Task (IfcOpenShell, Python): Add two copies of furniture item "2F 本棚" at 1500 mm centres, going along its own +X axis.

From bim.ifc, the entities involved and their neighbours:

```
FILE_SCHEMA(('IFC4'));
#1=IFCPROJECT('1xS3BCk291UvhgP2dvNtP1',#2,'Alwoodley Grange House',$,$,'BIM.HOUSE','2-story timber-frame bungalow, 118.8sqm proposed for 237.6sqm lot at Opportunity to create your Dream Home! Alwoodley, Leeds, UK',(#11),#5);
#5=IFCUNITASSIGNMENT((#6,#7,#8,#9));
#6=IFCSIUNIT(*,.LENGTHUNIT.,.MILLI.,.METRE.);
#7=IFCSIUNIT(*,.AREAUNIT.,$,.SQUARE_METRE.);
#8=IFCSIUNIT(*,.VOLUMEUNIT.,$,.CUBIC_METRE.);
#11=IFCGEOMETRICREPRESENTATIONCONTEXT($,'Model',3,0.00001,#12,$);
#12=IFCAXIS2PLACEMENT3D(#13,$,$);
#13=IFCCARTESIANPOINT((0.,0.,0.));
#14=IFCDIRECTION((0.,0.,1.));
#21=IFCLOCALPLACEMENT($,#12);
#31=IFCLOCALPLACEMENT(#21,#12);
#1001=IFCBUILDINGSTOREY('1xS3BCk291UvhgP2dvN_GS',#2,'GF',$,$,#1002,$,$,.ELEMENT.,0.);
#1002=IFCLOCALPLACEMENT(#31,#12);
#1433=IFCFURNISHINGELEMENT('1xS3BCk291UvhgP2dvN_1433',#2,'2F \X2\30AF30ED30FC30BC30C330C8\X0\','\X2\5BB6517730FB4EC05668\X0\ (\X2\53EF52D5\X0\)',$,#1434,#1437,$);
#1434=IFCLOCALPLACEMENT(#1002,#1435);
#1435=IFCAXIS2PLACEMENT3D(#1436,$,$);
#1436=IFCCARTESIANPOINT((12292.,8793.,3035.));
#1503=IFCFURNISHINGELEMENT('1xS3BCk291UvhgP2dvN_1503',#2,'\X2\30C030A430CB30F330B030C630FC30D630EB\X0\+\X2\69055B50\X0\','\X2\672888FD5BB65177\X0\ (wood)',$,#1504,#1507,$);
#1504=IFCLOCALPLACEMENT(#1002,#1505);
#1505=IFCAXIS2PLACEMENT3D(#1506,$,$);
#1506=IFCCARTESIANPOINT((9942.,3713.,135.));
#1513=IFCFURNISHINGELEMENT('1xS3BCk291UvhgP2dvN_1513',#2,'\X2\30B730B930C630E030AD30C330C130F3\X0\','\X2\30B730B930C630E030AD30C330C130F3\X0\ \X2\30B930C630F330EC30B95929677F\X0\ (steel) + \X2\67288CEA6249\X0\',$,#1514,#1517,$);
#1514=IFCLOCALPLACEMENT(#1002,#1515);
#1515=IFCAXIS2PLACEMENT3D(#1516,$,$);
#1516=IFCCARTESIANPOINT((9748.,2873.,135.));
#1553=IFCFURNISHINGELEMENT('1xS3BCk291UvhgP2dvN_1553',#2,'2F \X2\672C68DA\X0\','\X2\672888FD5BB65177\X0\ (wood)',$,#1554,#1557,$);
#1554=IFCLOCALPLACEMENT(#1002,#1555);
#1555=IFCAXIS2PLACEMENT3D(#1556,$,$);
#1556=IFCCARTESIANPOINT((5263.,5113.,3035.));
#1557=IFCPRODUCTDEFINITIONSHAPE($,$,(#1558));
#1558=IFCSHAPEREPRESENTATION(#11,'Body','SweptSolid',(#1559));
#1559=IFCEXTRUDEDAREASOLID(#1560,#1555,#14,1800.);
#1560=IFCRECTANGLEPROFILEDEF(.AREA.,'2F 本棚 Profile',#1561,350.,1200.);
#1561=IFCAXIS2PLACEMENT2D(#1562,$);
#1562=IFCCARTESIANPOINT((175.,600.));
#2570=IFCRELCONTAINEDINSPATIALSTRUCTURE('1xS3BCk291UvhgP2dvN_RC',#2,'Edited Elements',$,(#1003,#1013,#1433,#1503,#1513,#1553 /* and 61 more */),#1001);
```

```python
import ifcopenshell
import ifcopenshell.api.geometry
import ifcopenshell.api.root
import ifcopenshell.util.element
import ifcopenshell.util.placement

model = ifcopenshell.open("bim.ifc")


def reuse_history(source, copy):
    """copy_class also copies each property set's owner history, people and application; keep the originals."""
    for rel in copy.IsDefinedBy:
        if rel.is_a("IfcRelDefinesByProperties") and (history := rel.RelatingPropertyDefinition.OwnerHistory):
            rel.RelatingPropertyDefinition.OwnerHistory = source.OwnerHistory
            ifcopenshell.util.element.remove_deep2(model, history)


source = model.by_guid("1xS3BCk291UvhgP2dvN_1553")
base = ifcopenshell.util.placement.get_local_placement(source.ObjectPlacement)
step = base[:3, 0] * 1500.0

for i in range(1, 3):
    copy = ifcopenshell.api.root.copy_class(model, product=source)
    copy.Representation = ifcopenshell.util.element.copy_deep(
        model, source.Representation, exclude=["IfcGeometricRepresentationContext", "IfcRepresentationMap"]
    )
    reuse_history(source, copy)
    matrix = base.copy()
    matrix[:3, 3] += i * step
    print("added at", matrix[:3, 3].round(3) + 0.0)
    ifcopenshell.api.geometry.edit_object_placement(model, product=copy, matrix=matrix, is_si=False)

model.write("bim_updated.ifc")
```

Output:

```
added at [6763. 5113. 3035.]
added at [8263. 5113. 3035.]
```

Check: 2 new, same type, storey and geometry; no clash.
